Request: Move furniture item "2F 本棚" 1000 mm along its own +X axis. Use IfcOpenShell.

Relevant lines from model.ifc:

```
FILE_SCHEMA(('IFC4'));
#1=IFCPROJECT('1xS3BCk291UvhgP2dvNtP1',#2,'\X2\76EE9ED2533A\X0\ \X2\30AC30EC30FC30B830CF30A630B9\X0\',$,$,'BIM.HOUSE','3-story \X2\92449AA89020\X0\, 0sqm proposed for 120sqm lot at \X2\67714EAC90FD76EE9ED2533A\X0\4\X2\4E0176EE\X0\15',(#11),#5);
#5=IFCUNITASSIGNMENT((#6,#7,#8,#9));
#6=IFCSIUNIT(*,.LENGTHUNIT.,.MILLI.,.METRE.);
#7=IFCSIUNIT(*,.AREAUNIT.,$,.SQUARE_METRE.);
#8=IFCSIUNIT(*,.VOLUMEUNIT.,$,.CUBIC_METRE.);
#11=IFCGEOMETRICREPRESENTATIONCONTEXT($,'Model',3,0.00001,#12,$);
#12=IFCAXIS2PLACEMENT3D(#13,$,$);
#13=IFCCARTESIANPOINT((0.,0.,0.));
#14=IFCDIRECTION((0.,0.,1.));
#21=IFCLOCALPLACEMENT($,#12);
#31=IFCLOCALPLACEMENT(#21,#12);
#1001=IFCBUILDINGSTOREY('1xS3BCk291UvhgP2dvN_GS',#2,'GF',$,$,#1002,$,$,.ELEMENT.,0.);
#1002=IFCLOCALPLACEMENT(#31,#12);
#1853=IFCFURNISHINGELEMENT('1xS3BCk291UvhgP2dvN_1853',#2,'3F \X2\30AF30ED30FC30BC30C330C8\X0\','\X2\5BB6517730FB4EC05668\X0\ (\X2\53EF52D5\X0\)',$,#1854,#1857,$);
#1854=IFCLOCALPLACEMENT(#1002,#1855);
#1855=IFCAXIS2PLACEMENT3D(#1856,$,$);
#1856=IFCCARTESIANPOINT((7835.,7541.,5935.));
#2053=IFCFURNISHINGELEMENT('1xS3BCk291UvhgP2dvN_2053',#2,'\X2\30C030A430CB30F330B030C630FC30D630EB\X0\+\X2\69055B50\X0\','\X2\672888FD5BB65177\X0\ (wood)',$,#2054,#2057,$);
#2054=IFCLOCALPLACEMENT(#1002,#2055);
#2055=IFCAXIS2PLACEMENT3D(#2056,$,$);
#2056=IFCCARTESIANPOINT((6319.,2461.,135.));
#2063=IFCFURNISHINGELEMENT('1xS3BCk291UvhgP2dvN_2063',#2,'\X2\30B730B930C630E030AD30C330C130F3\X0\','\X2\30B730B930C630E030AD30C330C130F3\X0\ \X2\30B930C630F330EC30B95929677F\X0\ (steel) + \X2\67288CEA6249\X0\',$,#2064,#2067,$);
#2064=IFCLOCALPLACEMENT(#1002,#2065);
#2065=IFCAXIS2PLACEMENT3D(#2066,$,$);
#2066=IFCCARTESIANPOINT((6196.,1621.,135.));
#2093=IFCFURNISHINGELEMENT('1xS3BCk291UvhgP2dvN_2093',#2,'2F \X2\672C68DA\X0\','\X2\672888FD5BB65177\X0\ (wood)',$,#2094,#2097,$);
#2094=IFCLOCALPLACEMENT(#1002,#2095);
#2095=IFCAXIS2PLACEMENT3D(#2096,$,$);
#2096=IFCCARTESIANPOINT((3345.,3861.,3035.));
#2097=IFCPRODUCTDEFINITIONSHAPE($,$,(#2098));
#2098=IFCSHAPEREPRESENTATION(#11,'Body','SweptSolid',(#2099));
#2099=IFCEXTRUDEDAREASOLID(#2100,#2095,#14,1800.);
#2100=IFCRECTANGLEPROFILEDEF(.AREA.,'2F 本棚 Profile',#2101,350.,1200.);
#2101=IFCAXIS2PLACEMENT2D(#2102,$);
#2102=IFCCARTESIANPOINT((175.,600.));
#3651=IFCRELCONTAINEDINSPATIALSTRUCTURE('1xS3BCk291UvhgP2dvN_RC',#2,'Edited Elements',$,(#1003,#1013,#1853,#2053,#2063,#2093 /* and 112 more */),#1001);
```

```python
import ifcopenshell
import ifcopenshell.api.geometry
import ifcopenshell.util.placement

model = ifcopenshell.open("model.ifc")

item = model.by_guid("1xS3BCk291UvhgP2dvN_2093")
matrix = ifcopenshell.util.placement.get_local_placement(item.ObjectPlacement)
matrix[:3, 3] += matrix[:3, 0] * 1000.0
ifcopenshell.api.geometry.edit_object_placement(model, product=item, matrix=matrix, is_si=False)

print(ifcopenshell.util.placement.get_local_placement(item.ObjectPlacement).round(3) + 0.0)

model.write("model-out.ifc")
```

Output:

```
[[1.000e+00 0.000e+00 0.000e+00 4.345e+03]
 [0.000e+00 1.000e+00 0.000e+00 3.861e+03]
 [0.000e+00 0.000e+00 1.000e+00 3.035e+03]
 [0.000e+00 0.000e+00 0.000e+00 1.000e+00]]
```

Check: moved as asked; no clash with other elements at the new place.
